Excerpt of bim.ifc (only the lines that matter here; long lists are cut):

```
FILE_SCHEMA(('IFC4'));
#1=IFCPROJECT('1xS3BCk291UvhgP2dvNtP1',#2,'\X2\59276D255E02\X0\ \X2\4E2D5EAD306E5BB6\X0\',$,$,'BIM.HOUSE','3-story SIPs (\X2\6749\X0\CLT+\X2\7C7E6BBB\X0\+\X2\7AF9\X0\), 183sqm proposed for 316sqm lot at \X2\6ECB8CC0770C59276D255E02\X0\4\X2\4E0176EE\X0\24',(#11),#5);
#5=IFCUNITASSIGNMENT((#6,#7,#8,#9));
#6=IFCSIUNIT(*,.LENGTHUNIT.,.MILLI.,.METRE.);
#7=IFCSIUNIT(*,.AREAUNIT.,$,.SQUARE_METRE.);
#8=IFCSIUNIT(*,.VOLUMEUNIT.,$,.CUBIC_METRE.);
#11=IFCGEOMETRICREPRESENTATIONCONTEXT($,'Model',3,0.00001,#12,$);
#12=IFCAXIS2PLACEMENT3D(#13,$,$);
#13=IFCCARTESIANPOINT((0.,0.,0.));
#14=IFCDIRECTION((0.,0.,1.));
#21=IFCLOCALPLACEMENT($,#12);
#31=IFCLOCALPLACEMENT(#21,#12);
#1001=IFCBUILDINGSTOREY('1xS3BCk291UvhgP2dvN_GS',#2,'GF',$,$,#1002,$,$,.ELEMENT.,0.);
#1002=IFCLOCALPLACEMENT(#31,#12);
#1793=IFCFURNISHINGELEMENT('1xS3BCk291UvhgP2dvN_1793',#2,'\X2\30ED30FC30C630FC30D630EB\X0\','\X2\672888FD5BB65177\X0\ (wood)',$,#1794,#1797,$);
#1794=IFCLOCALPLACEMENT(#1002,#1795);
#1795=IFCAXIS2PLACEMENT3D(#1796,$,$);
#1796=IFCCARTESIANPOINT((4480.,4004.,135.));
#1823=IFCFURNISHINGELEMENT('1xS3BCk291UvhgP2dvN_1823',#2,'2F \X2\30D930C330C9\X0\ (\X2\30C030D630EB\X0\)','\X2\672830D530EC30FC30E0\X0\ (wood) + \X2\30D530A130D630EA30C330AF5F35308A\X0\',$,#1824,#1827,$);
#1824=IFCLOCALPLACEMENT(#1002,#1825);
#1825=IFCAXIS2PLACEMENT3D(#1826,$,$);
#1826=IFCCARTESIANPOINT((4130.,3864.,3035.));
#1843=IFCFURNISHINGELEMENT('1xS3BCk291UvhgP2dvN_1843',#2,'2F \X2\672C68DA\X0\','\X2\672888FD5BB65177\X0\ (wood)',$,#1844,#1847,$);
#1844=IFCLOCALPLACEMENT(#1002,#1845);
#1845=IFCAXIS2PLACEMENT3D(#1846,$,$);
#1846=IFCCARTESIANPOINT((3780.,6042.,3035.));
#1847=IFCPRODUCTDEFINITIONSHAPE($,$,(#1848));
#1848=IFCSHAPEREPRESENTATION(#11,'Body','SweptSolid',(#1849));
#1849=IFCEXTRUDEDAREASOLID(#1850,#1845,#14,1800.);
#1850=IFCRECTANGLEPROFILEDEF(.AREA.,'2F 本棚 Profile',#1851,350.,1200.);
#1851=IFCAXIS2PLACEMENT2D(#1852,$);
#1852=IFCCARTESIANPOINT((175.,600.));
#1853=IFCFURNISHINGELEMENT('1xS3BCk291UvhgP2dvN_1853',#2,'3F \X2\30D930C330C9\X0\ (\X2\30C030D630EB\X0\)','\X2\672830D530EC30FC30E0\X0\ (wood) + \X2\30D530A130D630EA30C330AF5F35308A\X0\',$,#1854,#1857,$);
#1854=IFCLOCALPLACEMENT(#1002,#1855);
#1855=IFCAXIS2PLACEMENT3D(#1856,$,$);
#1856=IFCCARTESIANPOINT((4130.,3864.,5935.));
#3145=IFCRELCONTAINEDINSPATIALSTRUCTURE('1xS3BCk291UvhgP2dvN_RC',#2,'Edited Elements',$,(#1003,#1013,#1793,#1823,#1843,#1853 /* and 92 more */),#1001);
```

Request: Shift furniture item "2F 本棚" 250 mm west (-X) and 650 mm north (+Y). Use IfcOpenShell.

```python
import ifcopenshell
import ifcopenshell.api.geometry
import ifcopenshell.util.placement

model = ifcopenshell.open("bim.ifc")

item = model.by_guid("1xS3BCk291UvhgP2dvN_1843")
matrix = ifcopenshell.util.placement.get_local_placement(item.ObjectPlacement)
matrix[0, 3] -= 250.0
matrix[1, 3] += 650.0
ifcopenshell.api.geometry.edit_object_placement(model, product=item, matrix=matrix, is_si=False)

print(ifcopenshell.util.placement.get_local_placement(item.ObjectPlacement).round(3) + 0.0)

model.write("bim-out.ifc")
```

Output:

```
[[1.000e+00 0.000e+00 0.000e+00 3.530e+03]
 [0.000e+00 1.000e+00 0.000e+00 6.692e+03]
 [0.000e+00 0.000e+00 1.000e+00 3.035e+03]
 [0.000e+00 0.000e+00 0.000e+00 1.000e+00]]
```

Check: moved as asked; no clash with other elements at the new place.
